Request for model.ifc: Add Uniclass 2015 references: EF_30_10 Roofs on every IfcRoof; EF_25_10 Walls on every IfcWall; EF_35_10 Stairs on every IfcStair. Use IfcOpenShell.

First a look at what the model holds.

```python
import ifcopenshell

model = ifcopenshell.open("model.ifc")
print(model.schema)
print("classifications:", [c.Name for c in model.by_type("IfcClassification")])
for ifc_class in ("IfcDoor", "IfcRoof", "IfcStair", "IfcWall", "IfcWindow"):
    print(ifc_class, len(model.by_type(ifc_class)))
```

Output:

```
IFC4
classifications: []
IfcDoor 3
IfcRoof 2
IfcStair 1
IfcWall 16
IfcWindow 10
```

```python
import ifcopenshell
import ifcopenshell.api.classification

model = ifcopenshell.open("model.ifc")

system = ifcopenshell.api.classification.add_classification(model, classification="Uniclass 2015")

codes = {
    "IfcRoof": ("EF_30_10", "Roofs"),
    "IfcWall": ("EF_25_10", "Walls"),
    "IfcStair": ("EF_35_10", "Stairs"),
}
for ifc_class, (code, name) in codes.items():
    products = model.by_type(ifc_class)
    ifcopenshell.api.classification.add_reference(
        model, products=products, classification=system, identification=code, name=name
    )
    print(code, len(products))

model.write("model_rev.ifc")
```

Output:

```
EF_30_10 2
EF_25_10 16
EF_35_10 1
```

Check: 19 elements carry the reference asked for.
